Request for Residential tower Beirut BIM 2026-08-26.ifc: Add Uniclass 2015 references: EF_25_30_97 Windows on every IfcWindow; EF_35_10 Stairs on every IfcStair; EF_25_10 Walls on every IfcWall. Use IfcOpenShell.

First a look at what the model holds.

```python
import ifcopenshell

model = ifcopenshell.open("Residential tower Beirut BIM 2026-08-26.ifc")
print(model.schema)
print("classifications:", [c.Name for c in model.by_type("IfcClassification")])
for ifc_class in ("IfcDoor", "IfcRoof", "IfcStair", "IfcWall", "IfcWindow"):
    print(ifc_class, len(model.by_type(ifc_class)))
```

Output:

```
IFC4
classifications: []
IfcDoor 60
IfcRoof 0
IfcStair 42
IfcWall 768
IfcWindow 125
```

```python
import ifcopenshell
import ifcopenshell.api.classification

model = ifcopenshell.open("Residential tower Beirut BIM 2026-08-26.ifc")

system = ifcopenshell.api.classification.add_classification(model, classification="Uniclass 2015")

codes = {
    "IfcWindow": ("EF_25_30_97", "Windows"),
    "IfcStair": ("EF_35_10", "Stairs"),
    "IfcWall": ("EF_25_10", "Walls"),
}
for ifc_class, (code, name) in codes.items():
    products = model.by_type(ifc_class)
    ifcopenshell.api.classification.add_reference(
        model, products=products, classification=system, identification=code, name=name
    )
    print(code, len(products))

model.write("Residential tower Beirut BIM 2026-08-26_rev.ifc")
```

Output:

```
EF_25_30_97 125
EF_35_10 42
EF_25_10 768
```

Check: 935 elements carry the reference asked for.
